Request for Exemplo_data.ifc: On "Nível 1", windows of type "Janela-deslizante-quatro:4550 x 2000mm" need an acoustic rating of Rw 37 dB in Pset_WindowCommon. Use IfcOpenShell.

First a look at what the model holds.

```python
import ifcopenshell
import ifcopenshell.util.element

model = ifcopenshell.open("Exemplo_data.ifc")
print(model.schema)
storey = next(s for s in model.by_type("IfcBuildingStorey") if s.Name == "Nível 1")
windows = [e for e in ifcopenshell.util.element.get_decomposition(storey) if e.is_a("IfcWindow")]
seen = {}
for e in windows:
    element_type = ifcopenshell.util.element.get_type(e)
    key = (element_type.Name if element_type != e and element_type else None, ifcopenshell.util.element.get_pset(e, "Pset_WindowCommon", "AcousticRating"))
    seen[key] = seen.get(key, 0) + 1
for (name, value), count in sorted(seen.items(), key=str):
    print(count, "x", name, "|", value)
```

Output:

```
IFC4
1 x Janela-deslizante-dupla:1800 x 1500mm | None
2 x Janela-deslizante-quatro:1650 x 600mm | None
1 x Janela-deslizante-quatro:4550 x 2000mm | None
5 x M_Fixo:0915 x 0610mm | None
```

```python
import ifcopenshell
import ifcopenshell.api.pset
import ifcopenshell.util.element

model = ifcopenshell.open("Exemplo_data.ifc")

storey = next(s for s in model.by_type("IfcBuildingStorey") if s.Name == "Nível 1")
windows = [e for e in ifcopenshell.util.element.get_decomposition(storey) if e.is_a("IfcWindow")]

count = 0
for e in windows:
    element_type = ifcopenshell.util.element.get_type(e)
    if element_type in (None, e) or element_type.Name != "Janela-deslizante-quatro:4550 x 2000mm":
        continue
    # add_pset returns the element's existing set when there is one.
    pset = ifcopenshell.api.pset.add_pset(model, product=e, name="Pset_WindowCommon")
    ifcopenshell.api.pset.edit_pset(model, pset=pset, properties={"AcousticRating": "Rw 37 dB"})
    count += 1

print(count, "windows updated")

model.write("Exemplo_data-out.ifc")
```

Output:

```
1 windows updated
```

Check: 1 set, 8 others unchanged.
